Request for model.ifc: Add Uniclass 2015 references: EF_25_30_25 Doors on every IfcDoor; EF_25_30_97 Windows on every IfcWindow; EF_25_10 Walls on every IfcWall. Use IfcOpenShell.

First a look at what the model holds.

```python
import ifcopenshell

model = ifcopenshell.open("model.ifc")
print(model.schema)
print("classifications:", [c.Name for c in model.by_type("IfcClassification")])
for ifc_class in ("IfcDoor", "IfcRoof", "IfcStair", "IfcWall", "IfcWindow"):
    print(ifc_class, len(model.by_type(ifc_class)))
```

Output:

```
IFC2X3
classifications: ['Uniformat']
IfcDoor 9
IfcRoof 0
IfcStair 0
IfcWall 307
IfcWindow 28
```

```python
import ifcopenshell
import ifcopenshell.api.classification

model = ifcopenshell.open("model.ifc")

# IFC2X3 requires Source and Edition and has no link from the project to the system.
system = model.create_entity("IfcClassification", Source="NBS", Edition="2015", Name="Uniclass 2015")

codes = {
    "IfcDoor": ("EF_25_30_25", "Doors"),
    "IfcWindow": ("EF_25_30_97", "Windows"),
    "IfcWall": ("EF_25_10", "Walls"),
}
for ifc_class, (code, name) in codes.items():
    products = model.by_type(ifc_class)
    ifcopenshell.api.classification.add_reference(
        model, products=products, classification=system, identification=code, name=name
    )
    print(code, len(products))

model.write("model_updated.ifc")
```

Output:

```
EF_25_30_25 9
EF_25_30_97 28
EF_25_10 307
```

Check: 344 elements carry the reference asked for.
